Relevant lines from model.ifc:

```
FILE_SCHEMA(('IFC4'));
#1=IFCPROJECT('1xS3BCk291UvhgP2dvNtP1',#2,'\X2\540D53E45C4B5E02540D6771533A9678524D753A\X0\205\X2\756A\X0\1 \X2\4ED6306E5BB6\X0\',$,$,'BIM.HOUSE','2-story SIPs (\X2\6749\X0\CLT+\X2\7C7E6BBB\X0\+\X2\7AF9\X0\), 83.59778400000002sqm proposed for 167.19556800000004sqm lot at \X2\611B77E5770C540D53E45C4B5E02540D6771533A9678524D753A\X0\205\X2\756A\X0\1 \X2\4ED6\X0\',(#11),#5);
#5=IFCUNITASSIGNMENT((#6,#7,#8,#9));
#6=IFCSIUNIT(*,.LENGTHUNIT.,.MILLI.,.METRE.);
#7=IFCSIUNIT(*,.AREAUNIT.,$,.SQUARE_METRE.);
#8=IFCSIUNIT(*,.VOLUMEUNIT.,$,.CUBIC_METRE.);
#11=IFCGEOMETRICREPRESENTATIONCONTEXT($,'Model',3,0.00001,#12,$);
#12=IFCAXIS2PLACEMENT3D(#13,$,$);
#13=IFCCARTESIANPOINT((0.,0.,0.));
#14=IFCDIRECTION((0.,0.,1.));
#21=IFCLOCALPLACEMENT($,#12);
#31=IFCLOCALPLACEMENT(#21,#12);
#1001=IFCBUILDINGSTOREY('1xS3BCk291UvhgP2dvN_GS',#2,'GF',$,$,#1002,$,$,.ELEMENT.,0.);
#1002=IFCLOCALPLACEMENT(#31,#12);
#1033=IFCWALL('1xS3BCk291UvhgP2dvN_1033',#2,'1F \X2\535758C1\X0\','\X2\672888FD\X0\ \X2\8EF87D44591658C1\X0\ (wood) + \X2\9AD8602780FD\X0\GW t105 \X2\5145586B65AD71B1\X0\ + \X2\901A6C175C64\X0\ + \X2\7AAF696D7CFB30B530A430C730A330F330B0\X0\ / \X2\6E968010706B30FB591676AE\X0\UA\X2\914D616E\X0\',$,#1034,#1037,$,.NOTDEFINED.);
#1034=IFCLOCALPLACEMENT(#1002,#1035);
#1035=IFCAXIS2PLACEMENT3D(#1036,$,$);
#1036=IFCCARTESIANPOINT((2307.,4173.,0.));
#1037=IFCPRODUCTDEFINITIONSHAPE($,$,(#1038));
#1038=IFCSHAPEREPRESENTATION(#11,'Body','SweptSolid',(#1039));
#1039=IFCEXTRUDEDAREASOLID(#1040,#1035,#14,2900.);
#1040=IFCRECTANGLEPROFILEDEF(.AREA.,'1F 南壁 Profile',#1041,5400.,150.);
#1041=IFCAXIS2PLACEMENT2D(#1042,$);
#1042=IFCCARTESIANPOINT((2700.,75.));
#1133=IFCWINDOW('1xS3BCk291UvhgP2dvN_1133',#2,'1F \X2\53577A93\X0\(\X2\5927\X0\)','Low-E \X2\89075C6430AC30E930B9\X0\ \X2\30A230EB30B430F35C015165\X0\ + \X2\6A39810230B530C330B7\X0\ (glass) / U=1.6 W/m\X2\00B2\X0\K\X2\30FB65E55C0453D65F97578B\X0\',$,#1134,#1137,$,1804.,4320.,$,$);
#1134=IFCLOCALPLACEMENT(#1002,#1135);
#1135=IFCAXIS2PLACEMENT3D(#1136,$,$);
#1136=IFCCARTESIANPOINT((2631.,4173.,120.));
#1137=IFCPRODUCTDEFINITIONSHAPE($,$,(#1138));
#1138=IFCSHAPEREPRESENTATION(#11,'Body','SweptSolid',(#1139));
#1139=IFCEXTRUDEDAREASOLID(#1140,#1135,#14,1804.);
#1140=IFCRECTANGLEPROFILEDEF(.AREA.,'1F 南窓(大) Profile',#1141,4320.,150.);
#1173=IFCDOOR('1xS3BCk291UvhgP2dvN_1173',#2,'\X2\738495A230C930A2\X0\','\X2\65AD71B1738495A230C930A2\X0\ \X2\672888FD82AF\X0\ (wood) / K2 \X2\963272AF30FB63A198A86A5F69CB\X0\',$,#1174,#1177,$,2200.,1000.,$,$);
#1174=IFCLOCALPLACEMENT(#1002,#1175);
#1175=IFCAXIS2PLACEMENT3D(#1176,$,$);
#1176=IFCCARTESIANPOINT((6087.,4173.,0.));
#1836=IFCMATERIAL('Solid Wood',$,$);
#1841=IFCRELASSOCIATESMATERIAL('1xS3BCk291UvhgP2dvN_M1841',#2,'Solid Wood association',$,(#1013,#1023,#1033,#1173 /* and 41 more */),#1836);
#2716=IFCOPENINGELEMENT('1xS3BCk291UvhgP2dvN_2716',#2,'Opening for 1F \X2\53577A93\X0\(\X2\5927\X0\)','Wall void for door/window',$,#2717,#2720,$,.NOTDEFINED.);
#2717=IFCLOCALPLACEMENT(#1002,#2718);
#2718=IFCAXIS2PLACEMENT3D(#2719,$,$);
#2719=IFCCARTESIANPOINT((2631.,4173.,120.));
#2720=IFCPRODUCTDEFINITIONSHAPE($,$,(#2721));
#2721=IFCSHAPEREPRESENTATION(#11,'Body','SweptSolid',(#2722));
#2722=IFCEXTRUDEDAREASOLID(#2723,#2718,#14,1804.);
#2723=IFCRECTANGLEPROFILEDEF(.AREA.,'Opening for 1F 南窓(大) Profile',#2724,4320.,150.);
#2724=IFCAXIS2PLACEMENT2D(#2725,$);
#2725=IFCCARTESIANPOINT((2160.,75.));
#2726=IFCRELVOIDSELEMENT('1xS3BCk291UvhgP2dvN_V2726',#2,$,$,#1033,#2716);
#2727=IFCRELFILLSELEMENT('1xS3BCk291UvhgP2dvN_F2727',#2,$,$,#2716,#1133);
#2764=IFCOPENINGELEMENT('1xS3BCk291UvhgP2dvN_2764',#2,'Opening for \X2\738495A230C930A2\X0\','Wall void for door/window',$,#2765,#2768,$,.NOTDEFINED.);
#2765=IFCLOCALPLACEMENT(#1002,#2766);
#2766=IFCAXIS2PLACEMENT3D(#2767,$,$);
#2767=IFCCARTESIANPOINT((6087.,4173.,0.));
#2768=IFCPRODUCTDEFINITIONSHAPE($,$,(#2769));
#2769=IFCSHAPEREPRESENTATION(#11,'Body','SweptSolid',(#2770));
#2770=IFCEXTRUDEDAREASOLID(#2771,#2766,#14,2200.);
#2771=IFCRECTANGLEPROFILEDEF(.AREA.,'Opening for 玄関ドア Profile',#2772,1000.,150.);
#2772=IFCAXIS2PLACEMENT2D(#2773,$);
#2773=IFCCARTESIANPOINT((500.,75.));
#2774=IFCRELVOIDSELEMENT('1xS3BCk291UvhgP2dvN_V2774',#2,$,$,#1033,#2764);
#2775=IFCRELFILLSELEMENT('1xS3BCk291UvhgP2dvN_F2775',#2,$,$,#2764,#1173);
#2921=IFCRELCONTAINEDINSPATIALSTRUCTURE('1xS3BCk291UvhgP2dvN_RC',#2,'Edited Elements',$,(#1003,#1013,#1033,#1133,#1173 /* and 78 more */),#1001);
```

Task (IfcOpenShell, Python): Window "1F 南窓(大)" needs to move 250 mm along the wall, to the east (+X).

```python
import ifcopenshell
import ifcopenshell.api.geometry
import ifcopenshell.util.placement

model = ifcopenshell.open("model.ifc")

window = model.by_id(1133)
opening = window.FillsVoids[0].RelatingOpeningElement
wall = opening.VoidsElements[0].RelatingBuildingElement

wall_matrix = ifcopenshell.util.placement.get_local_placement(wall.ObjectPlacement)
shift = wall_matrix[:3, 0] * 250.0
before = ifcopenshell.util.placement.get_local_placement(window.ObjectPlacement)[:3, 3].copy()

# The window is not placed relative to its opening, so move both.
for product in (opening, window):
    matrix = ifcopenshell.util.placement.get_local_placement(product.ObjectPlacement)
    matrix[:3, 3] += shift
    ifcopenshell.api.geometry.edit_object_placement(model, product=product, matrix=matrix, is_si=False)

after = ifcopenshell.util.placement.get_local_placement(window.ObjectPlacement)[:3, 3]
print("window moved by", (after - before).round(3) + 0.0)

model.write("model_edited.ifc")
```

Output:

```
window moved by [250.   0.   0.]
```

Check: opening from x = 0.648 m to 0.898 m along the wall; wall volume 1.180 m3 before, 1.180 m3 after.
